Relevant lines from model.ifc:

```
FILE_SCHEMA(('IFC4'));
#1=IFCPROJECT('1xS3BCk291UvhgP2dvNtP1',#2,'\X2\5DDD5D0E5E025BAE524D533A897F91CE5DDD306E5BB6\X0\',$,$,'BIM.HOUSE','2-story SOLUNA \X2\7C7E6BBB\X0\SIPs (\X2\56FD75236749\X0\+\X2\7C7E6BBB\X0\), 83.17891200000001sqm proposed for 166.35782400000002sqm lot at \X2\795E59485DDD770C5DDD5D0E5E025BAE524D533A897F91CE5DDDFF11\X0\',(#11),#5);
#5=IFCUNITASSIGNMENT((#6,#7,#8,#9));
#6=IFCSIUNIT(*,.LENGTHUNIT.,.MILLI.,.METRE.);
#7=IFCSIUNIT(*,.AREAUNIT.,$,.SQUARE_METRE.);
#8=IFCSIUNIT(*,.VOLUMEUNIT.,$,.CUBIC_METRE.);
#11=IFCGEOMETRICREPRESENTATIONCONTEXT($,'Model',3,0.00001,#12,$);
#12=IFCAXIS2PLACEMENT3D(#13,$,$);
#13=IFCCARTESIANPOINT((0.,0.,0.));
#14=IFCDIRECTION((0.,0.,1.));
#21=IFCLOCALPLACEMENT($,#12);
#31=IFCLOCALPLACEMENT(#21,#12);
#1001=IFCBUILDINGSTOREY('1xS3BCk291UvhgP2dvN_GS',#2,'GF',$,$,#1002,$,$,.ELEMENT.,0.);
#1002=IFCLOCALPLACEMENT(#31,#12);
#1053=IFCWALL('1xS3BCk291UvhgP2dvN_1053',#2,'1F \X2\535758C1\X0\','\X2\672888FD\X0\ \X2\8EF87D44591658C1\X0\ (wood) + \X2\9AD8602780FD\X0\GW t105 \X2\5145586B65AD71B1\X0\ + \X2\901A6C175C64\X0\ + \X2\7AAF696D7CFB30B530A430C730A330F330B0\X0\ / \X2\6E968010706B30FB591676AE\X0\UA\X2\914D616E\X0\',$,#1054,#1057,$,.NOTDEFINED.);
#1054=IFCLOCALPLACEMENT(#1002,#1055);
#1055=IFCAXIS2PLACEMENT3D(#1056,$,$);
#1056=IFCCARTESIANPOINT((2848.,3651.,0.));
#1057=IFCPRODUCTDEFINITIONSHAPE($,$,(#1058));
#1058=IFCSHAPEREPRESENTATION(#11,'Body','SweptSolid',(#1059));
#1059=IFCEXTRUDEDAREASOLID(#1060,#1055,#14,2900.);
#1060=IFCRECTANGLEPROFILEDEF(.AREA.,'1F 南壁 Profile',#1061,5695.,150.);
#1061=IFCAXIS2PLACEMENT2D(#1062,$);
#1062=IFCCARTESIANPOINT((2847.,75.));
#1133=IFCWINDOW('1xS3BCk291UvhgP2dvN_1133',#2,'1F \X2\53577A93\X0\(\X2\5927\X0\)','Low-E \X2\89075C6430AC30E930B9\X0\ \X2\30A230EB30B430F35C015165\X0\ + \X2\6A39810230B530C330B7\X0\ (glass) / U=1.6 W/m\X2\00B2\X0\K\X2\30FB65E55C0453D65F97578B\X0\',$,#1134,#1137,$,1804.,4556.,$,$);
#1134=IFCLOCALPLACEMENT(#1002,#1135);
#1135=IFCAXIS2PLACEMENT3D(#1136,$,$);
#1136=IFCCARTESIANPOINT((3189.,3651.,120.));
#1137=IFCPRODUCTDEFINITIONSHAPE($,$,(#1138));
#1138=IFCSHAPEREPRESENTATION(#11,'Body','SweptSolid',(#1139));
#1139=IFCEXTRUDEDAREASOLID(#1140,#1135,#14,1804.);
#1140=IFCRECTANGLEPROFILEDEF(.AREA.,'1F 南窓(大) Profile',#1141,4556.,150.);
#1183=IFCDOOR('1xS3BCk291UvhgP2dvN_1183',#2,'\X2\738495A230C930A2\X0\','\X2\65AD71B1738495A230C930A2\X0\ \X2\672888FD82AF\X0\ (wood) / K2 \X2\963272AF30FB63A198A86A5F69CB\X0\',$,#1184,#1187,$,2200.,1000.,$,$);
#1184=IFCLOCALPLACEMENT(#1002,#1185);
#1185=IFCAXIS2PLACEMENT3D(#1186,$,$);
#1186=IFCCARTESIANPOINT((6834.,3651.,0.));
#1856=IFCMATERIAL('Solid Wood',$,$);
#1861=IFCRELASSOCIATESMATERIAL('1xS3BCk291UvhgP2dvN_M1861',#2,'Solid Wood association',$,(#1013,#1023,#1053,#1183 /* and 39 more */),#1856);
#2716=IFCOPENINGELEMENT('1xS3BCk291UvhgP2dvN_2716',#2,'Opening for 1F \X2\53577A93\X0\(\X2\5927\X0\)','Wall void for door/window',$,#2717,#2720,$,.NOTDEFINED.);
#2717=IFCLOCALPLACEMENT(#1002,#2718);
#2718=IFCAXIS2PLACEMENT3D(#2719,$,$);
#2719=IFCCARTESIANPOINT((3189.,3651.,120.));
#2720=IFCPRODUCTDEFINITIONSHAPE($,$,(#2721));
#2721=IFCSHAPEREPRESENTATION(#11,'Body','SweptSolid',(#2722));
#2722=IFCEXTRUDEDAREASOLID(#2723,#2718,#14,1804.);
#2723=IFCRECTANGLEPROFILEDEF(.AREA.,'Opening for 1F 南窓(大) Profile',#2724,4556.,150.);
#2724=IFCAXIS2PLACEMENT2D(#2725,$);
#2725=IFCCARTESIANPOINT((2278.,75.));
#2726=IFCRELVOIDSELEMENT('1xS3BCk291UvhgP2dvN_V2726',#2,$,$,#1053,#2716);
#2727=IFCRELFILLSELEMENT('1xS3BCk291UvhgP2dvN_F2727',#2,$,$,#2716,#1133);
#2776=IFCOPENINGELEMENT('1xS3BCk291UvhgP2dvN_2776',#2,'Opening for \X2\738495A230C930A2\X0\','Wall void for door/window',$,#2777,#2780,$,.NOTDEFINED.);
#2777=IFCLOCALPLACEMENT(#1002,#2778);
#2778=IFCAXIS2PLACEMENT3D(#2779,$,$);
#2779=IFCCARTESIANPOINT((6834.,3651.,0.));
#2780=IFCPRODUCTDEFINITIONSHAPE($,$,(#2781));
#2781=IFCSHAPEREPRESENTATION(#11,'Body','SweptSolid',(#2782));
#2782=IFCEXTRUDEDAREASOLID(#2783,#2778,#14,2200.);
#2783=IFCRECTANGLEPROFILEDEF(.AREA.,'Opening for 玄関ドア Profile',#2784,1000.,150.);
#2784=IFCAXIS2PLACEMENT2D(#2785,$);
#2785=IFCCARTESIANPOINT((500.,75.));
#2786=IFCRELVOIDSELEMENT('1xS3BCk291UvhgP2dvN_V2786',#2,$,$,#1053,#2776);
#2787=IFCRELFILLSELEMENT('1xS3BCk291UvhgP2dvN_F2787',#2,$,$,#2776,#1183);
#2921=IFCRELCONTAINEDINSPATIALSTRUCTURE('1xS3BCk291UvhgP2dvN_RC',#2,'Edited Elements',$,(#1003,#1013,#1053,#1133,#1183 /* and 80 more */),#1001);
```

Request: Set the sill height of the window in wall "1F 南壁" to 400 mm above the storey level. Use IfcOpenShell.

```python
import numpy as np
import ifcopenshell
import ifcopenshell.api.geometry
import ifcopenshell.geom
import ifcopenshell.util.element
import ifcopenshell.util.placement
import ifcopenshell.util.shape
import ifcopenshell.util.unit

model = ifcopenshell.open("model.ifc")
unit_scale = ifcopenshell.util.unit.calculate_unit_scale(model)

window = model.by_id(1133)
opening = window.FillsVoids[0].RelatingOpeningElement
storey = ifcopenshell.util.element.get_container(window, ifc_class="IfcBuildingStorey")
level = ifcopenshell.util.placement.get_local_placement(storey.ObjectPlacement)[2, 3]

# The opening's origin need not be at the sill, so measure its lowest point.
shape = ifcopenshell.geom.create_shape(ifcopenshell.geom.settings(), opening)
bottom = ifcopenshell.util.shape.get_shape_bottom_elevation(shape, shape.geometry) / unit_scale
dz = level + 0.4 / unit_scale - bottom

shift = np.array([0.0, 0.0, dz])
# The window is not placed relative to its opening, so move both.
for product in (opening, window):
    matrix = ifcopenshell.util.placement.get_local_placement(product.ObjectPlacement)
    matrix[:3, 3] += shift
    ifcopenshell.api.geometry.edit_object_placement(model, product=product, matrix=matrix, is_si=False)

print(f"moved by {dz * unit_scale:+.3f} m")

model.write("model_edited.ifc")
```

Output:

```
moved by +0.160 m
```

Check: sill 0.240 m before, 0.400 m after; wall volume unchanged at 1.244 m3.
